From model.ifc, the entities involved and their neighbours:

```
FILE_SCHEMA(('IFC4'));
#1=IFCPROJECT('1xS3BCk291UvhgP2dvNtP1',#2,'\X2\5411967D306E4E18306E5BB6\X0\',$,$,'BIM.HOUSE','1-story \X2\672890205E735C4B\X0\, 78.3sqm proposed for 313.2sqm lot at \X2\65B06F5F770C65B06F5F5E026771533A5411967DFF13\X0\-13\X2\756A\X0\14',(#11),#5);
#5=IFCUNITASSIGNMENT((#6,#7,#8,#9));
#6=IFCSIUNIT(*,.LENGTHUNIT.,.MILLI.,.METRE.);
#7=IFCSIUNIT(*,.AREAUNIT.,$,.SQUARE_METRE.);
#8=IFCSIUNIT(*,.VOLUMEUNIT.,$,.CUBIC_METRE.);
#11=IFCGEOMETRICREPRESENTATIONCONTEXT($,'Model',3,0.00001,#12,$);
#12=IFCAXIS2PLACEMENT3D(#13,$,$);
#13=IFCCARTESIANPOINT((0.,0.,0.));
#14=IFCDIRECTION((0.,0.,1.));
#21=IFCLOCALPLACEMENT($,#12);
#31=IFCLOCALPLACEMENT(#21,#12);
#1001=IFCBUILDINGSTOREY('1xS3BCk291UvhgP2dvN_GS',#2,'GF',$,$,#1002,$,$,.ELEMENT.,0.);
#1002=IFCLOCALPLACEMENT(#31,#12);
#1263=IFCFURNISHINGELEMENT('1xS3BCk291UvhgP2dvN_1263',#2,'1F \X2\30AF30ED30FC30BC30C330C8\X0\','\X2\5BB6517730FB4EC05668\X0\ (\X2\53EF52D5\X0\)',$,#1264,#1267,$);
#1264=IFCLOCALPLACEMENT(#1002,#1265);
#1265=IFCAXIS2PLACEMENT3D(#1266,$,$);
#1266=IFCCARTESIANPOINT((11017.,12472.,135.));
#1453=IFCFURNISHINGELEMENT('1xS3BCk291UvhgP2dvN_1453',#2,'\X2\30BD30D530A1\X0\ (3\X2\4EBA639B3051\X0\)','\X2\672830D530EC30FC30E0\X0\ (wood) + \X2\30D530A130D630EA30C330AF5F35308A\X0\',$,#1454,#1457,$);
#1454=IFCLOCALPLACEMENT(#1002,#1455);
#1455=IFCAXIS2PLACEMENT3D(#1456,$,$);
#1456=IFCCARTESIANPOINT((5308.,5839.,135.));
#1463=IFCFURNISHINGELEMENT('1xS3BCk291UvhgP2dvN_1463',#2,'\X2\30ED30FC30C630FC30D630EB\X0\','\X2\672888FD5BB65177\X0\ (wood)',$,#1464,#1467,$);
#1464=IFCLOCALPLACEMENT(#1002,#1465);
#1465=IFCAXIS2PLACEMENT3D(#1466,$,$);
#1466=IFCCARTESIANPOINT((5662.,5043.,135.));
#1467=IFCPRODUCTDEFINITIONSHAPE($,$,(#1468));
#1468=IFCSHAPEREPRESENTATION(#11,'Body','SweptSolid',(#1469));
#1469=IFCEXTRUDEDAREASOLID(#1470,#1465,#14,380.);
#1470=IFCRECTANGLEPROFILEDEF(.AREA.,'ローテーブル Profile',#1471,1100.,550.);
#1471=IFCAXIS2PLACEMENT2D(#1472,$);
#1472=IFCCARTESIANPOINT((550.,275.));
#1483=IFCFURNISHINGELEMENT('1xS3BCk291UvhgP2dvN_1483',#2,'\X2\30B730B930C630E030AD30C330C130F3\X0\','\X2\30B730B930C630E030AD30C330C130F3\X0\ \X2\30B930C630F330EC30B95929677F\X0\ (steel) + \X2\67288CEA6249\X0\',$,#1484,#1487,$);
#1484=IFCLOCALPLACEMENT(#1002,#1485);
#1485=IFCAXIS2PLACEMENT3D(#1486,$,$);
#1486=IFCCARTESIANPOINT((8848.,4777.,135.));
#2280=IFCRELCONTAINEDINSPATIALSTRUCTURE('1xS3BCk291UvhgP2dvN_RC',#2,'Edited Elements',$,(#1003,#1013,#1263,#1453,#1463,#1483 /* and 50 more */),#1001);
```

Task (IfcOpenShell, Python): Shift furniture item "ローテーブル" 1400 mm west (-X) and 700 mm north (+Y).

```python
import ifcopenshell
import ifcopenshell.api.geometry
import ifcopenshell.util.placement

model = ifcopenshell.open("model.ifc")

item = model.by_guid("1xS3BCk291UvhgP2dvN_1463")
matrix = ifcopenshell.util.placement.get_local_placement(item.ObjectPlacement)
matrix[0, 3] -= 1400.0
matrix[1, 3] += 700.0
ifcopenshell.api.geometry.edit_object_placement(model, product=item, matrix=matrix, is_si=False)

print(ifcopenshell.util.placement.get_local_placement(item.ObjectPlacement).round(3) + 0.0)

model.write("model_v2.ifc")
```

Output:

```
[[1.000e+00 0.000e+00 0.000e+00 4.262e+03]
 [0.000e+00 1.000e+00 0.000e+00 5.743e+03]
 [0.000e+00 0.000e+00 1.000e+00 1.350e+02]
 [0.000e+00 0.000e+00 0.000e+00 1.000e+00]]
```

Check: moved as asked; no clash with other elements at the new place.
